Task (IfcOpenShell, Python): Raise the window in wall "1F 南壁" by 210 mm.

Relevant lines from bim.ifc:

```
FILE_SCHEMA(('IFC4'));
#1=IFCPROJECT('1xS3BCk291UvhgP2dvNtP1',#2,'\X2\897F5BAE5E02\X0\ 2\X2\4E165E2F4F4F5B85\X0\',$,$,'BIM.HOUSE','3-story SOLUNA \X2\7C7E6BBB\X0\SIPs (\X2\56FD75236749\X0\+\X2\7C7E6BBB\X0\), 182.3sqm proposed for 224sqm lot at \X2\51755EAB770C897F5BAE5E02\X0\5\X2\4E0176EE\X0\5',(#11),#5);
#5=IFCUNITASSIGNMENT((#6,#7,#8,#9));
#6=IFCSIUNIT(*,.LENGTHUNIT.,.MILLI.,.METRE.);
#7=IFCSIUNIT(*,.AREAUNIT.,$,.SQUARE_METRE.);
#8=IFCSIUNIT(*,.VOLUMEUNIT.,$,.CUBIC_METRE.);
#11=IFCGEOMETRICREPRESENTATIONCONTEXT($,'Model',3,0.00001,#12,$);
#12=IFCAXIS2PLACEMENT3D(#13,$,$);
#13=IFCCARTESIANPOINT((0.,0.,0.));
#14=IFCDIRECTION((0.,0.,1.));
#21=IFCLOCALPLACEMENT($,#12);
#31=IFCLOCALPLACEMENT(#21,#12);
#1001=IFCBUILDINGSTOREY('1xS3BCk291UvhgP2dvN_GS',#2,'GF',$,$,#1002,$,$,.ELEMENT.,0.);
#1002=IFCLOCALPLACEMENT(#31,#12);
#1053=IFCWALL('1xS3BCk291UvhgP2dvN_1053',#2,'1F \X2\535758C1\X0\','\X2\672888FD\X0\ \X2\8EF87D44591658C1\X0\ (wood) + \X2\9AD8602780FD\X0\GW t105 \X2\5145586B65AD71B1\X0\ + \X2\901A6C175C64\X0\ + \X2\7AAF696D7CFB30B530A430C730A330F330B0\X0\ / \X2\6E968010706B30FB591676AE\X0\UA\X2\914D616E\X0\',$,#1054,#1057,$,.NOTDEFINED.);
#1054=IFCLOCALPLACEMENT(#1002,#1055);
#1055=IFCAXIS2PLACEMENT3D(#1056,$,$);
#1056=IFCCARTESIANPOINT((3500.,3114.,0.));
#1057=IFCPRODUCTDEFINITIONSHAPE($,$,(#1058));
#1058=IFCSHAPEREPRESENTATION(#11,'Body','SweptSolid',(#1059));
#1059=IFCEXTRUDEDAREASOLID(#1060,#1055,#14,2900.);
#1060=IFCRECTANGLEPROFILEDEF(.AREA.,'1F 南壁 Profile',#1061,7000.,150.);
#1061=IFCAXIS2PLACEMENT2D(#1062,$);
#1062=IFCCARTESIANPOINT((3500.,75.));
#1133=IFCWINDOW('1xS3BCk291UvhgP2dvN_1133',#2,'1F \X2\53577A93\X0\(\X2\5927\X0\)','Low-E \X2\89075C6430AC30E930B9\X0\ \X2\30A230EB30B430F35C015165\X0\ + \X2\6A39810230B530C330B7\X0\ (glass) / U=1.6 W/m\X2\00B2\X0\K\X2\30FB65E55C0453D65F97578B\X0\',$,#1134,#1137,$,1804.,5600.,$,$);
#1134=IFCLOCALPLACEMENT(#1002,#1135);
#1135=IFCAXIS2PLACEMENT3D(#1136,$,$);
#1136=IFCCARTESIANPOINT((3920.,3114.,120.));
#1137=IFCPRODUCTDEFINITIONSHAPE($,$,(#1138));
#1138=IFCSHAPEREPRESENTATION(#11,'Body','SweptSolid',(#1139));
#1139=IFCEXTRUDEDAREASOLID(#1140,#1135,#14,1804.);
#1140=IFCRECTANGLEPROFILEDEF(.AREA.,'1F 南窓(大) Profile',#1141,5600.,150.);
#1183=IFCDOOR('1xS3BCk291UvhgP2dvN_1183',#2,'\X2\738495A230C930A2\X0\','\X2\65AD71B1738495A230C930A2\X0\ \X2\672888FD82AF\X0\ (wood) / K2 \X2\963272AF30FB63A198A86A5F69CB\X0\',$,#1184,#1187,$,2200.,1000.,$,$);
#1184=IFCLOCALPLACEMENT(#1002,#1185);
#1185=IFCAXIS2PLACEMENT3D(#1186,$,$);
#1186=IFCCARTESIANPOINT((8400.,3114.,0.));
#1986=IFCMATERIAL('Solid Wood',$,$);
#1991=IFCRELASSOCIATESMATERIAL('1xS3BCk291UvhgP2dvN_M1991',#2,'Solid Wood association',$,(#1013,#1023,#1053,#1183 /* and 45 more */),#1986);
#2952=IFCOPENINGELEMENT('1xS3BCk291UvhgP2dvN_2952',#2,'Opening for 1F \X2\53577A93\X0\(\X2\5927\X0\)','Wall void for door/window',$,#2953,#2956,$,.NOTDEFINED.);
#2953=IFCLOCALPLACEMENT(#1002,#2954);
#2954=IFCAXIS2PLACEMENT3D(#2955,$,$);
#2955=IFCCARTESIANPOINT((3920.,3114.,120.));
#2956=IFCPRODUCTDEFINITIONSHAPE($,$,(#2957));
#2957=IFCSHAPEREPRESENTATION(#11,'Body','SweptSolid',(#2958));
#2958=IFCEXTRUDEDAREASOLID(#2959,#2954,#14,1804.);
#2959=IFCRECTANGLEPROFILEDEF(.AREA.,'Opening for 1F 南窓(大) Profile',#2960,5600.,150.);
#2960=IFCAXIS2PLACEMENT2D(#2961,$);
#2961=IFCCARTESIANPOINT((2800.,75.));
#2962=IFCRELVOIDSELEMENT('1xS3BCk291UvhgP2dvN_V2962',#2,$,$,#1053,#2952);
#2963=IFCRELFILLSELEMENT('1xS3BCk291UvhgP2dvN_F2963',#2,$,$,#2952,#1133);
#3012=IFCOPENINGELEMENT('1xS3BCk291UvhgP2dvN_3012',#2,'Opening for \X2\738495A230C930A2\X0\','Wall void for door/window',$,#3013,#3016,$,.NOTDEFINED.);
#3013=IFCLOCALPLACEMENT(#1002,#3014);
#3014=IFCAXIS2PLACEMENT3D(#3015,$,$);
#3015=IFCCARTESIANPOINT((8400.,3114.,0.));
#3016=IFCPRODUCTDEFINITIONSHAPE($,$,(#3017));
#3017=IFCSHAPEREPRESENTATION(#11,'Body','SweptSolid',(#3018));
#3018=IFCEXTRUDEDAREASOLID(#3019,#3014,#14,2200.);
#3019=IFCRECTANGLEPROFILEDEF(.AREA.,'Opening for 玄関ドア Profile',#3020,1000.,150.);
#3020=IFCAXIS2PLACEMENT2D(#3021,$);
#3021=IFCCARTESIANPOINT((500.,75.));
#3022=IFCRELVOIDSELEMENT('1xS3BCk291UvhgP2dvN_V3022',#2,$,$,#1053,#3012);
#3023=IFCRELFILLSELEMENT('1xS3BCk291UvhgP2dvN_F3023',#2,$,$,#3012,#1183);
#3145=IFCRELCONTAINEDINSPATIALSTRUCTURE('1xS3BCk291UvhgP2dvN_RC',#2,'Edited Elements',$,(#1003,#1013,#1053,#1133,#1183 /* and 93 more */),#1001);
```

```python
import numpy as np
import ifcopenshell
import ifcopenshell.api.geometry
import ifcopenshell.util.placement
import ifcopenshell.util.unit

model = ifcopenshell.open("bim.ifc")
unit_scale = ifcopenshell.util.unit.calculate_unit_scale(model)

window = model.by_guid("1xS3BCk291UvhgP2dvN_1133")
opening = window.FillsVoids[0].RelatingOpeningElement
dz = 210.0

shift = np.array([0.0, 0.0, dz])
# The window is not placed relative to its opening, so move both.
for product in (opening, window):
    matrix = ifcopenshell.util.placement.get_local_placement(product.ObjectPlacement)
    matrix[:3, 3] += shift
    ifcopenshell.api.geometry.edit_object_placement(model, product=product, matrix=matrix, is_si=False)

print(f"moved by {dz * unit_scale:+.3f} m")

model.write("bim_rev.ifc")
```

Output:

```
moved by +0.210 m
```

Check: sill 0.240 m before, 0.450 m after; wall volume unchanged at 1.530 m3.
